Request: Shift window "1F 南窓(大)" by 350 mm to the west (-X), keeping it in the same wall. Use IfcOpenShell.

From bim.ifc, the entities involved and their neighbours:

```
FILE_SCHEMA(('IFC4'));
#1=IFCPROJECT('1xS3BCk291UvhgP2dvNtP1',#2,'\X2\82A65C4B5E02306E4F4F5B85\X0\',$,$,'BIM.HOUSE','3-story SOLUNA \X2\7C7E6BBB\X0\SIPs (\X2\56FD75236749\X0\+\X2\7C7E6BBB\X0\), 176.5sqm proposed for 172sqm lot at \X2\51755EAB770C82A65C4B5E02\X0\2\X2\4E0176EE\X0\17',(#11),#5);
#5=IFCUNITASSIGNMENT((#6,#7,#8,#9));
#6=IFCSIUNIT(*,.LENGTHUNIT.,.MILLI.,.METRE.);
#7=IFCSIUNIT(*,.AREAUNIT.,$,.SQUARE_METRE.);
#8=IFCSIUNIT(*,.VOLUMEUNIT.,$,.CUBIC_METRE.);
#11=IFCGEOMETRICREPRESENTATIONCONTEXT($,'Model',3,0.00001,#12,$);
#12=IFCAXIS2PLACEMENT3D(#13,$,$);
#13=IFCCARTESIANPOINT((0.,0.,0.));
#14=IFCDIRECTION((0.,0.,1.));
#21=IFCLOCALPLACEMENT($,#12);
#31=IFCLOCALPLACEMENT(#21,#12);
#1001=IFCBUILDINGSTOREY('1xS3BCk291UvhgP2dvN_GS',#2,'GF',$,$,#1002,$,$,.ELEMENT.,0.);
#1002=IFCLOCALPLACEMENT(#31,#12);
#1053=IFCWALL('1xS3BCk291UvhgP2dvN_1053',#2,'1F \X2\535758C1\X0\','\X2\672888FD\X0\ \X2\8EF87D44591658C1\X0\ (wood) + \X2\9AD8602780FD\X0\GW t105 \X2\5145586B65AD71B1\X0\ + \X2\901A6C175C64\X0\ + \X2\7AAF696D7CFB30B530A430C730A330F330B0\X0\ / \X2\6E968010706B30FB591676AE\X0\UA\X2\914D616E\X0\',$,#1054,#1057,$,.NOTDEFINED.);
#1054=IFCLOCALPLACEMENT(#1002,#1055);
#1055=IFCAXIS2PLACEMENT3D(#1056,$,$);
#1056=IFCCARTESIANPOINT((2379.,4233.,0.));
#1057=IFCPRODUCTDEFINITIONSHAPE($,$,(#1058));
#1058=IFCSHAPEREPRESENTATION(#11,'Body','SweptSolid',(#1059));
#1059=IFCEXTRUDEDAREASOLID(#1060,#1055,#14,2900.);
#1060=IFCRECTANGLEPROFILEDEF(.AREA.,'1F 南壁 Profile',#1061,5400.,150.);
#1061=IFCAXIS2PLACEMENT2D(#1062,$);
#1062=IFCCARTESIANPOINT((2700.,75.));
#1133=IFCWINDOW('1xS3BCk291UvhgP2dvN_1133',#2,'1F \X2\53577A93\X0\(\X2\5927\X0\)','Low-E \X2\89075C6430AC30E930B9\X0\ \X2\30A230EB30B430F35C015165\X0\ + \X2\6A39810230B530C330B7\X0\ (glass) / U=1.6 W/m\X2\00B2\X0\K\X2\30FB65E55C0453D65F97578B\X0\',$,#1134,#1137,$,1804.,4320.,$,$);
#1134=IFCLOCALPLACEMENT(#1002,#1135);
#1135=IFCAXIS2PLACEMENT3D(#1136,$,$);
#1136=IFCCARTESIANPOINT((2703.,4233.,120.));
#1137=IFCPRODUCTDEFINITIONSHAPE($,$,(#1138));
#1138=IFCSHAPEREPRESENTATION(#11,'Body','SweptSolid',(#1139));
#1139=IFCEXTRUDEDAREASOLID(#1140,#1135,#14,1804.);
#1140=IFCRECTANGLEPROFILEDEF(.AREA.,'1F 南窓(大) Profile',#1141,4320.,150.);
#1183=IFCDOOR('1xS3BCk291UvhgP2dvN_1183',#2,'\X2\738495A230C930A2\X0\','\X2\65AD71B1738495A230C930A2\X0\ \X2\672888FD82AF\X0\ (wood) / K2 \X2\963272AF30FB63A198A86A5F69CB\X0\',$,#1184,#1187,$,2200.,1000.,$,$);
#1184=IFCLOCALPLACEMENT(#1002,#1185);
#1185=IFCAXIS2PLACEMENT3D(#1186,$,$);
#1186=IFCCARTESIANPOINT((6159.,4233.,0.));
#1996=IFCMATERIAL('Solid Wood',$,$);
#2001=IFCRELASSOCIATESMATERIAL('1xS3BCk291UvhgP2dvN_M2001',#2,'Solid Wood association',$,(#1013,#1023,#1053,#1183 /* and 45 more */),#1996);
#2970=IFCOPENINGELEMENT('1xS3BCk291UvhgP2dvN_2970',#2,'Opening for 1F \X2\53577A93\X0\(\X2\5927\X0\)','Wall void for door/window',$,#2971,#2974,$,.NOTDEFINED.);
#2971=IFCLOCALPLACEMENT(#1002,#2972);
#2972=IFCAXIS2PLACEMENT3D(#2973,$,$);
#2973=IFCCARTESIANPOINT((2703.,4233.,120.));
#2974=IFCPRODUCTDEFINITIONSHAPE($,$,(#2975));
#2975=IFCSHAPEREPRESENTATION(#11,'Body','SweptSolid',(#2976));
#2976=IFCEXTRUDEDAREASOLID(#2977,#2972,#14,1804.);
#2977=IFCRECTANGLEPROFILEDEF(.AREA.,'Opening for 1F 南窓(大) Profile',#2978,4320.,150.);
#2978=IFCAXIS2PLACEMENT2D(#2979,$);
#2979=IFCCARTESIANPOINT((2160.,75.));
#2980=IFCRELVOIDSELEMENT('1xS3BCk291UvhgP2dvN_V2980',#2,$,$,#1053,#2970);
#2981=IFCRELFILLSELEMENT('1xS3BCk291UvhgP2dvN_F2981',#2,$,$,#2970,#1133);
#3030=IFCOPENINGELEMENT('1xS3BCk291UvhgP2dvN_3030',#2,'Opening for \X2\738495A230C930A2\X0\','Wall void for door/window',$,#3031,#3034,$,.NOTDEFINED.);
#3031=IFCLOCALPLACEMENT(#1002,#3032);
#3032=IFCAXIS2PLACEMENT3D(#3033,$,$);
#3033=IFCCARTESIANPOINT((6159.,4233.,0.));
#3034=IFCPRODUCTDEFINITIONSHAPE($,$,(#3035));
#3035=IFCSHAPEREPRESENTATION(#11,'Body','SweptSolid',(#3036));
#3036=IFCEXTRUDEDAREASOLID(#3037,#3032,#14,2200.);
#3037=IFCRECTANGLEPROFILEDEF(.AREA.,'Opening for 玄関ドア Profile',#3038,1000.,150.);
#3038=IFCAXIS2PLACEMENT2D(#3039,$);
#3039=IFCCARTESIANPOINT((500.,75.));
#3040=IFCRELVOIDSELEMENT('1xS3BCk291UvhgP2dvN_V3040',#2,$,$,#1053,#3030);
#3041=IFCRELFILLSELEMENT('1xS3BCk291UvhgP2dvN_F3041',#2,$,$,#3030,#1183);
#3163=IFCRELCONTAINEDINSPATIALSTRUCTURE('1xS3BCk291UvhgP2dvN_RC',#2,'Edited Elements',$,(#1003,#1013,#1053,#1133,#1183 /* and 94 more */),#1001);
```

```python
import ifcopenshell
import ifcopenshell.api.geometry
import ifcopenshell.util.placement
import ifcopenshell.util.unit

model = ifcopenshell.open("bim.ifc")
unit_scale = ifcopenshell.util.unit.calculate_unit_scale(model)

window = model.by_id(1133)
opening = window.FillsVoids[0].RelatingOpeningElement
wall = opening.VoidsElements[0].RelatingBuildingElement

wall_matrix = ifcopenshell.util.placement.get_local_placement(wall.ObjectPlacement)
shift = wall_matrix[:3, 0] * -0.35 / unit_scale
before = ifcopenshell.util.placement.get_local_placement(window.ObjectPlacement)[:3, 3].copy()

# The window is not placed relative to its opening, so move both.
for product in (opening, window):
    matrix = ifcopenshell.util.placement.get_local_placement(product.ObjectPlacement)
    matrix[:3, 3] += shift
    ifcopenshell.api.geometry.edit_object_placement(model, product=product, matrix=matrix, is_si=False)

after = ifcopenshell.util.placement.get_local_placement(window.ObjectPlacement)[:3, 3]
print("window moved by", (after - before).round(3) + 0.0)

model.write("bim_updated.ifc")
```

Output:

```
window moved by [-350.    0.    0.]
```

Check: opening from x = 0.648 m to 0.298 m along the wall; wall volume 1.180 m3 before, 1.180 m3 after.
